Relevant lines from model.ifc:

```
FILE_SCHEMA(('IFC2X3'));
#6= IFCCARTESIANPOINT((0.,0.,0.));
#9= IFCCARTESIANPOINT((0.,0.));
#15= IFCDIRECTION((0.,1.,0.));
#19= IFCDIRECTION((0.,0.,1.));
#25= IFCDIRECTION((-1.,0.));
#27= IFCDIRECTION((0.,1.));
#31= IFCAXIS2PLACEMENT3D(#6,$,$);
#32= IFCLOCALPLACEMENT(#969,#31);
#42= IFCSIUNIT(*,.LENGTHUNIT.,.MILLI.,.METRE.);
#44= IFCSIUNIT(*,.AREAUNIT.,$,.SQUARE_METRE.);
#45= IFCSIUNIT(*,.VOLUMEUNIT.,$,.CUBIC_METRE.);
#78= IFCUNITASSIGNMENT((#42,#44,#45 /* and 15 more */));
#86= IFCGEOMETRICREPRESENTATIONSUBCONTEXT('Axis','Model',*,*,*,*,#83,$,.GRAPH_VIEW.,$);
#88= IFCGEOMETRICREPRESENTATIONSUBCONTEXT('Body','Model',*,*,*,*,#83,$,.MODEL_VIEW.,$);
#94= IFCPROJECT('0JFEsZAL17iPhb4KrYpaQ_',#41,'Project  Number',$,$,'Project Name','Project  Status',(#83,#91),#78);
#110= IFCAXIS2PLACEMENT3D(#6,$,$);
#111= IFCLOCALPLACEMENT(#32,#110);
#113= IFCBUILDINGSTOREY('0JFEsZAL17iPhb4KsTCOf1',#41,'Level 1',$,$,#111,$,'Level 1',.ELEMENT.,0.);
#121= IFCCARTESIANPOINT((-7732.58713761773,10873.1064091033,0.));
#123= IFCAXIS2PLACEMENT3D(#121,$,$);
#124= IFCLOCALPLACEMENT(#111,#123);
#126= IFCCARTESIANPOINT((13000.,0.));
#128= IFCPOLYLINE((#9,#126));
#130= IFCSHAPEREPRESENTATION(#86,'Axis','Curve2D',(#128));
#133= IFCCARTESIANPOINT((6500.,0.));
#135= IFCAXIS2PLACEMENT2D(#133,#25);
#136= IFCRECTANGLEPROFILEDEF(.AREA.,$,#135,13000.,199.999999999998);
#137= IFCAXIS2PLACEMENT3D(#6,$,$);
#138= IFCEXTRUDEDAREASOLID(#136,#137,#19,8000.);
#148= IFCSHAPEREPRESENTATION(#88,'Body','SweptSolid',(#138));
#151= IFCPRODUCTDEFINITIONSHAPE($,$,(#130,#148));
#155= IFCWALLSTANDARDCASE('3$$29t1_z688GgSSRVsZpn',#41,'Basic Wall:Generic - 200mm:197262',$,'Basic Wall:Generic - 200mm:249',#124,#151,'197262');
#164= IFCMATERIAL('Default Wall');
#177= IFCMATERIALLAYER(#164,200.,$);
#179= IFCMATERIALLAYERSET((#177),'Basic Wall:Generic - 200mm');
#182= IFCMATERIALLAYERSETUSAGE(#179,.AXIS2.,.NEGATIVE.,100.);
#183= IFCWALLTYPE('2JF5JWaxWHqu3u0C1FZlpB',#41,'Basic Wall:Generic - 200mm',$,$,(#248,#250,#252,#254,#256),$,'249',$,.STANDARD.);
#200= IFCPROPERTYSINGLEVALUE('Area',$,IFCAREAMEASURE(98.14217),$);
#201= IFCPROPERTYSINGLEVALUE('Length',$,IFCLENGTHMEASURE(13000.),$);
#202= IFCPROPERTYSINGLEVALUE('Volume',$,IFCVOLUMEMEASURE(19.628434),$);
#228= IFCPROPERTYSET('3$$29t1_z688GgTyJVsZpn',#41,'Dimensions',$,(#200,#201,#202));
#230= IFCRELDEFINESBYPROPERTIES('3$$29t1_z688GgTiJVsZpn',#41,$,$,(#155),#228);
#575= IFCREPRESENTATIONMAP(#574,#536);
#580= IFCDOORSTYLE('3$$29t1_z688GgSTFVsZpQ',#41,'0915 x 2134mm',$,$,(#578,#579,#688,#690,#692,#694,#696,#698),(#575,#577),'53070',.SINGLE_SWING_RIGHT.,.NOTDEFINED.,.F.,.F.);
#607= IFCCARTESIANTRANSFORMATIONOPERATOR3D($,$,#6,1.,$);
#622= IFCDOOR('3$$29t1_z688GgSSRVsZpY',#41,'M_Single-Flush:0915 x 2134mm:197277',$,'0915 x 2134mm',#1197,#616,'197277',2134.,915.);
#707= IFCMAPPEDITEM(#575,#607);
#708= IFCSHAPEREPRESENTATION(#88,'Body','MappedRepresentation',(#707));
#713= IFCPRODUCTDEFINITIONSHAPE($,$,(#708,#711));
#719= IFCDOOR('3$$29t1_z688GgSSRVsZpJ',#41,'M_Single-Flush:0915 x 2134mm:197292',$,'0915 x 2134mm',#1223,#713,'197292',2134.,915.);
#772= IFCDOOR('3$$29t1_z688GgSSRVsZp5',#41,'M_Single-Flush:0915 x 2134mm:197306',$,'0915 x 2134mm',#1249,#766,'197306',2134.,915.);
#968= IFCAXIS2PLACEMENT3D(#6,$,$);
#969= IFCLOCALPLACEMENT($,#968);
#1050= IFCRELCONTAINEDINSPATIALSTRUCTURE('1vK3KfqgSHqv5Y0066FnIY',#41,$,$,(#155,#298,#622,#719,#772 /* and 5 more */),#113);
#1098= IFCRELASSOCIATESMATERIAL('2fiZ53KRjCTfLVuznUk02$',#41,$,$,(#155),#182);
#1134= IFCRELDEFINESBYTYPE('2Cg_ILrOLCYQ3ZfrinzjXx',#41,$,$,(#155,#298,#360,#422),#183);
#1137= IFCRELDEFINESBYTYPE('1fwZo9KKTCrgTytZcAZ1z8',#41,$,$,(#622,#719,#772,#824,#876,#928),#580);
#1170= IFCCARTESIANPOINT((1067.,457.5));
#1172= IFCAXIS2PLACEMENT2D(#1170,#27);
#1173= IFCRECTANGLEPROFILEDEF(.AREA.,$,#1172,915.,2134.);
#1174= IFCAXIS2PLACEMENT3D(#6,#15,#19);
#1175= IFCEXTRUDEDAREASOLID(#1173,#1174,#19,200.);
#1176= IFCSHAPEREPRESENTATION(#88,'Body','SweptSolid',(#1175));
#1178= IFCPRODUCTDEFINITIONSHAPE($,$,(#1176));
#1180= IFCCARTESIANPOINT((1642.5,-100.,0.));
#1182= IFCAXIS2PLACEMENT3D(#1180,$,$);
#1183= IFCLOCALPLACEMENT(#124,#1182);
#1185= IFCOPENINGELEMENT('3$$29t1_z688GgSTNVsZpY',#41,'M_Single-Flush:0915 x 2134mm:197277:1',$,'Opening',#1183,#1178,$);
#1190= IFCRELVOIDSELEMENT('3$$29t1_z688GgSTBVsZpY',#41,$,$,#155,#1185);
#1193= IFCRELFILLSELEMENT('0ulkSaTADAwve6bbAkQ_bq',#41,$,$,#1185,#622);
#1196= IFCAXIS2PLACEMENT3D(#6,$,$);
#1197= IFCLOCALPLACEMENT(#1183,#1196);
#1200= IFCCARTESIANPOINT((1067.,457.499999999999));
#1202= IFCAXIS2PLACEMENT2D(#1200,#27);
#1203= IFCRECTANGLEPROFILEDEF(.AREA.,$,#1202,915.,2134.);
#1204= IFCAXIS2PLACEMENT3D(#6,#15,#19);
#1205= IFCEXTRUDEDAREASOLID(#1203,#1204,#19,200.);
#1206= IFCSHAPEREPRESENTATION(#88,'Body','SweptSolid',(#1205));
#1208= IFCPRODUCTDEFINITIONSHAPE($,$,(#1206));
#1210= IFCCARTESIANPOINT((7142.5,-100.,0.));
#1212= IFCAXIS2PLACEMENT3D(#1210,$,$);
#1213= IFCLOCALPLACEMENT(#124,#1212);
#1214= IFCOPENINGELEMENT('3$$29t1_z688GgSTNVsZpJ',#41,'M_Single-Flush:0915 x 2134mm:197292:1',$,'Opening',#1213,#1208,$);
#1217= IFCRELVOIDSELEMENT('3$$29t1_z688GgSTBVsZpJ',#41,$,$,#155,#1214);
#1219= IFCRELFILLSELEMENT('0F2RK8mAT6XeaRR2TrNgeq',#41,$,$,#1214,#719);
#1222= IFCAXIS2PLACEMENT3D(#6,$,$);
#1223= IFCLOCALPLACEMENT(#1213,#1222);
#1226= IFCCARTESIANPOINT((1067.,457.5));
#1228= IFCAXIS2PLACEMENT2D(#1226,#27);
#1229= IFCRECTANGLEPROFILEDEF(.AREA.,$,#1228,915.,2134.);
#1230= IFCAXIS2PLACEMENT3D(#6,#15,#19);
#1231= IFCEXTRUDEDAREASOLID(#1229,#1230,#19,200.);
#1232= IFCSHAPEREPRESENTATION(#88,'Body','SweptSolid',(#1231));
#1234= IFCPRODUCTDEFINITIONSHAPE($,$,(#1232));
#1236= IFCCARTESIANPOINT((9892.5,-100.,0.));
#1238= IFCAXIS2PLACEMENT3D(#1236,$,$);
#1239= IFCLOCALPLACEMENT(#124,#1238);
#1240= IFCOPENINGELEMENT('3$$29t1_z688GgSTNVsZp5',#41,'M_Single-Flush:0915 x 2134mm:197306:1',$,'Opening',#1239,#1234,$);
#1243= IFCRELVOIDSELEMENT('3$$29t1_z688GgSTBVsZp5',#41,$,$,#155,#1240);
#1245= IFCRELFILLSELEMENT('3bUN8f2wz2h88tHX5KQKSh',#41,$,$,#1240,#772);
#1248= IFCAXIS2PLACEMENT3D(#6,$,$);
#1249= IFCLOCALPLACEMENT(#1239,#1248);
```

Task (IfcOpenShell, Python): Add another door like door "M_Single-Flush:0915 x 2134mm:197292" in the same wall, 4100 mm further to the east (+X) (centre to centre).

```python
import ifcopenshell
import ifcopenshell.api.feature
import ifcopenshell.api.geometry
import ifcopenshell.api.pset
import ifcopenshell.api.root
import ifcopenshell.geom
import ifcopenshell.util.element
import ifcopenshell.util.placement
import ifcopenshell.util.shape
import ifcopenshell.util.unit

model = ifcopenshell.open("model.ifc")
area_scale = ifcopenshell.util.unit.calculate_unit_scale(model, "AREAUNIT")
volume_scale = ifcopenshell.util.unit.calculate_unit_scale(model, "VOLUMEUNIT")
settings = ifcopenshell.geom.settings()


def volume(element):
    """Net volume in cubic metres, openings subtracted."""
    shape = ifcopenshell.geom.create_shape(settings, element)
    return ifcopenshell.util.shape.get_volume(shape.geometry)


def reuse_history(source, copy):
    """copy_class also copies each property set's owner history, people and application; keep the originals."""
    for rel in copy.IsDefinedBy:
        if rel.is_a("IfcRelDefinesByProperties") and (history := rel.RelatingPropertyDefinition.OwnerHistory):
            rel.RelatingPropertyDefinition.OwnerHistory = source.OwnerHistory
            ifcopenshell.util.element.remove_deep2(model, history)


door = model.by_guid("3$$29t1_z688GgSSRVsZpJ")
opening = door.FillsVoids[0].RelatingOpeningElement
wall = opening.VoidsElements[0].RelatingBuildingElement
before = volume(wall)
shift = ifcopenshell.util.placement.get_local_placement(wall.ObjectPlacement)[:3, 0] * 4100.0

# copy_class copies the void relationship, type, container and properties, but no geometry.
new_opening = ifcopenshell.api.root.copy_class(model, product=opening)
new_opening.Representation = ifcopenshell.util.element.copy_deep(
    model, opening.Representation, exclude=["IfcGeometricRepresentationContext", "IfcRepresentationMap"]
)
new_opening.Name = "M_Single-Flush:0915 x 2134mm"
new_door = ifcopenshell.api.root.copy_class(model, product=door)
new_door.Representation = ifcopenshell.util.element.copy_deep(
    model, door.Representation, exclude=["IfcGeometricRepresentationContext", "IfcRepresentationMap"]
)
new_door.Name = "M_Single-Flush:0915 x 2134mm"
new_door.Tag = None
reuse_history(door, new_door)
fills = ifcopenshell.api.feature.add_filling(model, opening=new_opening, element=new_door)
fills.OwnerHistory = new_door.OwnerHistory  # required in IFC2X3

for old, new in ((opening, new_opening), (door, new_door)):
    matrix = ifcopenshell.util.placement.get_local_placement(old.ObjectPlacement)
    matrix[:3, 3] += shift
    ifcopenshell.api.geometry.edit_object_placement(model, product=new, matrix=matrix, is_si=False)

after = volume(wall)
thickness = 0.2  # wall thickness in metres

# Update the wall's stored quantities.
pset = model.by_id(ifcopenshell.util.element.get_pset(wall, "Dimensions", should_inherit=False)["id"])
ifcopenshell.api.pset.edit_pset(model, pset=pset, properties={
    "Area": model.create_entity("IfcAreaMeasure", after / thickness / area_scale),
    "Volume": model.create_entity("IfcVolumeMeasure", after / volume_scale),
})

print(f"wall volume {before:.3f} -> {after:.3f} m3")

model.write("model_updated.ifc")
```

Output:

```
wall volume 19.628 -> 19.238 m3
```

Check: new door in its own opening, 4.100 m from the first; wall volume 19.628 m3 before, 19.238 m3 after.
